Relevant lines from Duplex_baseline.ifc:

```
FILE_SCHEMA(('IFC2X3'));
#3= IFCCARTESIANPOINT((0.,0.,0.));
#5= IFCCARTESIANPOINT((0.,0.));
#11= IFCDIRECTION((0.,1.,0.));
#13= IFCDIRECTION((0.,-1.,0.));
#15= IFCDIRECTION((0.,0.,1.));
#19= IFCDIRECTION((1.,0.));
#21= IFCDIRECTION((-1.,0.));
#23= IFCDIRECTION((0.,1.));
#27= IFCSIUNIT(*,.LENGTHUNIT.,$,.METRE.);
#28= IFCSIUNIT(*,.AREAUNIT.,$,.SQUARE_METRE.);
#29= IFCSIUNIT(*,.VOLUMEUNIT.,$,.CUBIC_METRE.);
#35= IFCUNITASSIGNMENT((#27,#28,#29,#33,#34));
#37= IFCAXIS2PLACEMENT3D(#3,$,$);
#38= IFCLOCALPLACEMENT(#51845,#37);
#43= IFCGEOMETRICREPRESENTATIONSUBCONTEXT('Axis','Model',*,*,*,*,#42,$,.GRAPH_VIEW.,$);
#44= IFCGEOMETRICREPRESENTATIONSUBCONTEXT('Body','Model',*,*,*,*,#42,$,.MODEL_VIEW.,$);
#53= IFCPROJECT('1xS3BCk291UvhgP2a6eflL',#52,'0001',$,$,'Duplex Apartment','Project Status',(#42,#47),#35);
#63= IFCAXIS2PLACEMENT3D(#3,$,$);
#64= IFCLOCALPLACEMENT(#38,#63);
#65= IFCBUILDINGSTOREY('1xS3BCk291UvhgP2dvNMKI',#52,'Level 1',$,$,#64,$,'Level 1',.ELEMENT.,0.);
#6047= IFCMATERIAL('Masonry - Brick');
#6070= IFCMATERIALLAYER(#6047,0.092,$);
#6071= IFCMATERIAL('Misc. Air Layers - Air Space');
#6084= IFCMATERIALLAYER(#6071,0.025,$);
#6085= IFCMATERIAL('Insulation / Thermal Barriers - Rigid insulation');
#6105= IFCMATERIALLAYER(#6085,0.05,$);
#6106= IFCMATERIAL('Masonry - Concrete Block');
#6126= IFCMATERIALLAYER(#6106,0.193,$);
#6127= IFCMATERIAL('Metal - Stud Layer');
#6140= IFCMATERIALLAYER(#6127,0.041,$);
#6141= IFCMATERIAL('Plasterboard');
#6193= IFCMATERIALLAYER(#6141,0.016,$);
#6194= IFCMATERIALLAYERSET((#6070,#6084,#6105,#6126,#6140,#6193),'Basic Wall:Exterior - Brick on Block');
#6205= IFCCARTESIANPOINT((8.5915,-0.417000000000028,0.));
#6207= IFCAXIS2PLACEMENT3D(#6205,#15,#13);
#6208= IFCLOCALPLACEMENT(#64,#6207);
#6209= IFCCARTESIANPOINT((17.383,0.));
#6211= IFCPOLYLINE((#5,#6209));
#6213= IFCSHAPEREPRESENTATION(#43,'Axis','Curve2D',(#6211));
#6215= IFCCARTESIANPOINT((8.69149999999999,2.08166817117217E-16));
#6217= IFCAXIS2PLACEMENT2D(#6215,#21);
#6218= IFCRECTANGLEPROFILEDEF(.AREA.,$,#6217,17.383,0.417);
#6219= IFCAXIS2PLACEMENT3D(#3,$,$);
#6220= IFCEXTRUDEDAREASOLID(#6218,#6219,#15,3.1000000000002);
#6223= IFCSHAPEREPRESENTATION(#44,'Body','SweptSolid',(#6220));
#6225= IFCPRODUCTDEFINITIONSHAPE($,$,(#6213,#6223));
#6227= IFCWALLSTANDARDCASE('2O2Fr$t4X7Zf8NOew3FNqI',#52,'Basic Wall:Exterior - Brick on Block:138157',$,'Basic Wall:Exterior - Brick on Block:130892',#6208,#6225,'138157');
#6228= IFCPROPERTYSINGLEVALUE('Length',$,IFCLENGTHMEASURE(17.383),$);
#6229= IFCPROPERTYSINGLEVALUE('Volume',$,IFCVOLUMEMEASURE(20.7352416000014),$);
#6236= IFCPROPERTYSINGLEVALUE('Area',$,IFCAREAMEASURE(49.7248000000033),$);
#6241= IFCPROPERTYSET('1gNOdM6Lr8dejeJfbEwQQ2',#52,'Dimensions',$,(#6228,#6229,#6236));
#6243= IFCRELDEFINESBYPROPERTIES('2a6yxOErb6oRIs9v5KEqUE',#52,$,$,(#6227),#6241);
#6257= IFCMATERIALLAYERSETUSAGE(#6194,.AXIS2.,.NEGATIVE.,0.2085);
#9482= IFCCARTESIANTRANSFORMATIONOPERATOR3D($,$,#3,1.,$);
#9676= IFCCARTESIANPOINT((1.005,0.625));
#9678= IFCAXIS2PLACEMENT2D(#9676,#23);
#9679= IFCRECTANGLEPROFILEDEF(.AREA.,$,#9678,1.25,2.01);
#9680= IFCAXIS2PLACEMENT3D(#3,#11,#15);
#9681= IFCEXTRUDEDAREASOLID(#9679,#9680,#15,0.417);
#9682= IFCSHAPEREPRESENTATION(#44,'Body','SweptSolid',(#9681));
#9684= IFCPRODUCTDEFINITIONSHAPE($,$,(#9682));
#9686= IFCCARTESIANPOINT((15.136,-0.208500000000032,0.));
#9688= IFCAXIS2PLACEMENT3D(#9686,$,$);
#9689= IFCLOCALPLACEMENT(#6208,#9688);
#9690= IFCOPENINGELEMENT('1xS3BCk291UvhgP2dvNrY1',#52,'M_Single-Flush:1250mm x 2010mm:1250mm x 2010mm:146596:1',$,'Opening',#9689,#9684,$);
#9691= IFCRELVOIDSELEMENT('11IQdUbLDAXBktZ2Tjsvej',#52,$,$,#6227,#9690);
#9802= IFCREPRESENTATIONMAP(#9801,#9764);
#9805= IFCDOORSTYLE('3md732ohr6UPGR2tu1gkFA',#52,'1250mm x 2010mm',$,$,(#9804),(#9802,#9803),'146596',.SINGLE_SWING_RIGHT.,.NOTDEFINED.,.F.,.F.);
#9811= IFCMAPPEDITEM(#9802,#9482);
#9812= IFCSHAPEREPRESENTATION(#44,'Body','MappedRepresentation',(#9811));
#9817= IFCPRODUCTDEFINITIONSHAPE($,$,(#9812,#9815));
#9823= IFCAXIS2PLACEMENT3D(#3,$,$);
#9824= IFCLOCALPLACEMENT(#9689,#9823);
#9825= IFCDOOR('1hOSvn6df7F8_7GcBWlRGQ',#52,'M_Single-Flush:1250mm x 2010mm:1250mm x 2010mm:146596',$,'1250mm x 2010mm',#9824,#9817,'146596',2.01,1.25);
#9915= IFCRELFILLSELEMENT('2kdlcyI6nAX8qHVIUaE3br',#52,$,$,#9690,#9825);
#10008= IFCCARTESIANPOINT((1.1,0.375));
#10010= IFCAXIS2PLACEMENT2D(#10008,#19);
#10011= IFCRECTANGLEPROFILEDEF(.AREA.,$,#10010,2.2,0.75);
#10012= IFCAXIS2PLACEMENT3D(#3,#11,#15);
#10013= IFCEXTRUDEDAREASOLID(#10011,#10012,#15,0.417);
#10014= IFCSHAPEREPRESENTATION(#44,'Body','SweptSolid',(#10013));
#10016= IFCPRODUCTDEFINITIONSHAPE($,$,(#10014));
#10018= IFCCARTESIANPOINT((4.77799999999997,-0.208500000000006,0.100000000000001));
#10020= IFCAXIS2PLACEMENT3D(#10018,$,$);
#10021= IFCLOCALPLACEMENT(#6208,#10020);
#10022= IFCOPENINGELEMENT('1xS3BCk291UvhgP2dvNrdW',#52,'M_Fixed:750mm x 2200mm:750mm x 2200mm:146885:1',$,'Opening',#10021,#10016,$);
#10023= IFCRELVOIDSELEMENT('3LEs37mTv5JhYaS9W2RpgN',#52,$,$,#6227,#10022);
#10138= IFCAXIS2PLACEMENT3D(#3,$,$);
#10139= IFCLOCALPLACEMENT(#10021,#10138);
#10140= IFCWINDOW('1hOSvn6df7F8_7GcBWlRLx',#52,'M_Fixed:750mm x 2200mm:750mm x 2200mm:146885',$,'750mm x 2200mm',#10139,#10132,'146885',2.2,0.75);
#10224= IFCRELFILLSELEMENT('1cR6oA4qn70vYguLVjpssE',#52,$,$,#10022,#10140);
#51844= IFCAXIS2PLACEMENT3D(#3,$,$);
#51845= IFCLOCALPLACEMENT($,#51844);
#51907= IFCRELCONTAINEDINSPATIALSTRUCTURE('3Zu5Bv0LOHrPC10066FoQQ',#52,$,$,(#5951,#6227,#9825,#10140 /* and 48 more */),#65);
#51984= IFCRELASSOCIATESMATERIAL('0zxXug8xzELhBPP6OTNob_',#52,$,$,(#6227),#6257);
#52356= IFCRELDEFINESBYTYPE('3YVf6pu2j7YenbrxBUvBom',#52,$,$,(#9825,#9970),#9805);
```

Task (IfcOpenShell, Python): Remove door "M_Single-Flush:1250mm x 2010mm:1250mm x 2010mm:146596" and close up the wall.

```python
import ifcopenshell
import ifcopenshell.api.feature
import ifcopenshell.api.pset
import ifcopenshell.api.root
import ifcopenshell.geom
import ifcopenshell.util.element
import ifcopenshell.util.shape
import ifcopenshell.util.unit

model = ifcopenshell.open("Duplex_baseline.ifc")
area_scale = ifcopenshell.util.unit.calculate_unit_scale(model, "AREAUNIT")
volume_scale = ifcopenshell.util.unit.calculate_unit_scale(model, "VOLUMEUNIT")
settings = ifcopenshell.geom.settings()


def volume(element):
    """Net volume in cubic metres, openings subtracted."""
    shape = ifcopenshell.geom.create_shape(settings, element)
    return ifcopenshell.util.shape.get_volume(shape.geometry)


door = model.by_id(9825)
opening = door.FillsVoids[0].RelatingOpeningElement
wall = opening.VoidsElements[0].RelatingBuildingElement
before = volume(wall)

ifcopenshell.api.root.remove_product(model, product=door)
ifcopenshell.api.feature.remove_feature(model, feature=opening)

after = volume(wall)
thickness = 0.417  # wall thickness in metres

# Update the wall's stored quantities.
pset = model.by_id(ifcopenshell.util.element.get_pset(wall, "Dimensions", should_inherit=False)["id"])
ifcopenshell.api.pset.edit_pset(model, pset=pset, properties={
    "Volume": model.create_entity("IfcVolumeMeasure", after / volume_scale),
    "Area": model.create_entity("IfcAreaMeasure", after / thickness / area_scale),
})

print(f"wall volume {before:.3f} -> {after:.3f} m3")

model.write("Duplex_baseline_edited.ifc")
```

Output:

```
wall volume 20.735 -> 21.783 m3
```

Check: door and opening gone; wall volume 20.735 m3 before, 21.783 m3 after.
